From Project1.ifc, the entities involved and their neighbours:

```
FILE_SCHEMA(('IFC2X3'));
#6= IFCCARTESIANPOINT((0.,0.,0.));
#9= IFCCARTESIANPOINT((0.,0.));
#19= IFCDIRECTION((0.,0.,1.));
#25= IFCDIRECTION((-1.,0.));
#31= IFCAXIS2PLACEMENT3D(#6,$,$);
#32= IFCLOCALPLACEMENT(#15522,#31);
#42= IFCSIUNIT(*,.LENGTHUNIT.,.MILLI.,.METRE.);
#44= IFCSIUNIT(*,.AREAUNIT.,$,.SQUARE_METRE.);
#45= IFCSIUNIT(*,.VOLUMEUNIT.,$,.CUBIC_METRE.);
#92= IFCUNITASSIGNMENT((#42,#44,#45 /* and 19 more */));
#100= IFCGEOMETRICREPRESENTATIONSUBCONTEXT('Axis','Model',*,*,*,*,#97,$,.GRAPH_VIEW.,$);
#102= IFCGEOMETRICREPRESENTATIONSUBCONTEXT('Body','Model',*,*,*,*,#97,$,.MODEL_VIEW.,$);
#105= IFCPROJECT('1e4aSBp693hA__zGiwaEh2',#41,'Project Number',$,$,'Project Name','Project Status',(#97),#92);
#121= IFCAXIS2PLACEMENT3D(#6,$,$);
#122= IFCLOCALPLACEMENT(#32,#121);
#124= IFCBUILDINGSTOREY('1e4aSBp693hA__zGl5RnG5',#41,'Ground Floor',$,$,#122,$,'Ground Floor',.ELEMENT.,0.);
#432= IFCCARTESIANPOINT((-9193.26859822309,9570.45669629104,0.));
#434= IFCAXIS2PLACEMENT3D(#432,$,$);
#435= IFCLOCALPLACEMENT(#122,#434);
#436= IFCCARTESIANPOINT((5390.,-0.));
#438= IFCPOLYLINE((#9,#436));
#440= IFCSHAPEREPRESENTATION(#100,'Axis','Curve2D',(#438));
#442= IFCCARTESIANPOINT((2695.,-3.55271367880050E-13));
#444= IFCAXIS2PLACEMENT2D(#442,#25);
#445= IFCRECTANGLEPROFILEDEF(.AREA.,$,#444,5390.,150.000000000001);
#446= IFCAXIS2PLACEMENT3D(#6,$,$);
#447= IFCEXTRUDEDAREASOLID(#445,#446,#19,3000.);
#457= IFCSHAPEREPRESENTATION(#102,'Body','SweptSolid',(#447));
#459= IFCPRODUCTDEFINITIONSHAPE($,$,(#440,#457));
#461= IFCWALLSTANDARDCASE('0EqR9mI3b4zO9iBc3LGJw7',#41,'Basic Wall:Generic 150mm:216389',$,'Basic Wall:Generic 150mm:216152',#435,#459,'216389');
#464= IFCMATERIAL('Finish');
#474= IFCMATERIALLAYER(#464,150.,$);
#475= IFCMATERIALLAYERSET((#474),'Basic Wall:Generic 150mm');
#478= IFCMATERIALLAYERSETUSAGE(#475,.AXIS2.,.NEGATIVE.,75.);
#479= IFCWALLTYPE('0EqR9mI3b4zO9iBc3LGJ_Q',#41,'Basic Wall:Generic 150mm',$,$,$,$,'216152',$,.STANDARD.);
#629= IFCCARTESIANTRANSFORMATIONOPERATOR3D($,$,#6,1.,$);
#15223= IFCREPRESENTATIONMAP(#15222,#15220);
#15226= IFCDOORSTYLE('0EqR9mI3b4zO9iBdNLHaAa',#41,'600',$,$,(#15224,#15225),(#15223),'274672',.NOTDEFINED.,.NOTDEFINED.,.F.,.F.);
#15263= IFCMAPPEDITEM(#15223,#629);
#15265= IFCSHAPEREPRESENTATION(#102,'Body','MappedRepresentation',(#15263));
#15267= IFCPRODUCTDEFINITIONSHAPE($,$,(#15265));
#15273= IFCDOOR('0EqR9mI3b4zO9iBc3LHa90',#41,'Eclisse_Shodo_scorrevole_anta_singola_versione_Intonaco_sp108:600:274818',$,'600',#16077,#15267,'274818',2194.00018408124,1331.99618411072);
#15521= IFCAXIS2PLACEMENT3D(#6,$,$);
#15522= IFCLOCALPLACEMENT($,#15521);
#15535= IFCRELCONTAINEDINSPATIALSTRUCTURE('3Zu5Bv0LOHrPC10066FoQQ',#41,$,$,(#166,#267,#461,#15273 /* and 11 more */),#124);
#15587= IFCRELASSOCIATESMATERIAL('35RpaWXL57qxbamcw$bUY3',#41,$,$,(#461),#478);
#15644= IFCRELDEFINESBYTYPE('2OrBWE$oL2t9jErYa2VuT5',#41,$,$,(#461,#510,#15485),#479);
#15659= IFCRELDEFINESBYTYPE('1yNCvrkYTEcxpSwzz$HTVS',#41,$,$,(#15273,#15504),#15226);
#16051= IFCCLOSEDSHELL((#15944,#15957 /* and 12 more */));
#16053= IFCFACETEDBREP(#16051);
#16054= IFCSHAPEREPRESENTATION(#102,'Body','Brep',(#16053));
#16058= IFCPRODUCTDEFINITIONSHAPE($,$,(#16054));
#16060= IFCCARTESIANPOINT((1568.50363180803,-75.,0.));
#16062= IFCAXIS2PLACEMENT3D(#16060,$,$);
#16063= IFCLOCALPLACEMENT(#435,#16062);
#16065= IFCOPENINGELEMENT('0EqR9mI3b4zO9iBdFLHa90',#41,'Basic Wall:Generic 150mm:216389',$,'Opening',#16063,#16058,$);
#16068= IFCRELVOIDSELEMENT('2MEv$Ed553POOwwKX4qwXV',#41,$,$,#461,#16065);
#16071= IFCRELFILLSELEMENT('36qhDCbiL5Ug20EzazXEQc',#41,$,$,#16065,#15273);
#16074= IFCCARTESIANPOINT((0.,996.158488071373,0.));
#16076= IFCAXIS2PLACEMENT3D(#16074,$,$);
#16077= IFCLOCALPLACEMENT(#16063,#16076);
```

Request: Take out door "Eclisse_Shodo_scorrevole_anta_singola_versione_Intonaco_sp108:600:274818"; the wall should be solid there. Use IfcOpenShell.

```python
import ifcopenshell
import ifcopenshell.api.feature
import ifcopenshell.api.root
import ifcopenshell.geom
import ifcopenshell.util.shape

model = ifcopenshell.open("Project1.ifc")
settings = ifcopenshell.geom.settings()


def volume(element):
    """Net volume in cubic metres, openings subtracted."""
    shape = ifcopenshell.geom.create_shape(settings, element)
    return ifcopenshell.util.shape.get_volume(shape.geometry)


door = model.by_guid("0EqR9mI3b4zO9iBc3LHa90")
opening = door.FillsVoids[0].RelatingOpeningElement
wall = opening.VoidsElements[0].RelatingBuildingElement
before = volume(wall)

ifcopenshell.api.root.remove_product(model, product=door)
ifcopenshell.api.feature.remove_feature(model, feature=opening)

after = volume(wall)

print(f"wall volume {before:.3f} -> {after:.3f} m3")

model.write("Project1-out.ifc")
```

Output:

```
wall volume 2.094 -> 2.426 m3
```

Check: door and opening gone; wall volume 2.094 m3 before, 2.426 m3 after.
